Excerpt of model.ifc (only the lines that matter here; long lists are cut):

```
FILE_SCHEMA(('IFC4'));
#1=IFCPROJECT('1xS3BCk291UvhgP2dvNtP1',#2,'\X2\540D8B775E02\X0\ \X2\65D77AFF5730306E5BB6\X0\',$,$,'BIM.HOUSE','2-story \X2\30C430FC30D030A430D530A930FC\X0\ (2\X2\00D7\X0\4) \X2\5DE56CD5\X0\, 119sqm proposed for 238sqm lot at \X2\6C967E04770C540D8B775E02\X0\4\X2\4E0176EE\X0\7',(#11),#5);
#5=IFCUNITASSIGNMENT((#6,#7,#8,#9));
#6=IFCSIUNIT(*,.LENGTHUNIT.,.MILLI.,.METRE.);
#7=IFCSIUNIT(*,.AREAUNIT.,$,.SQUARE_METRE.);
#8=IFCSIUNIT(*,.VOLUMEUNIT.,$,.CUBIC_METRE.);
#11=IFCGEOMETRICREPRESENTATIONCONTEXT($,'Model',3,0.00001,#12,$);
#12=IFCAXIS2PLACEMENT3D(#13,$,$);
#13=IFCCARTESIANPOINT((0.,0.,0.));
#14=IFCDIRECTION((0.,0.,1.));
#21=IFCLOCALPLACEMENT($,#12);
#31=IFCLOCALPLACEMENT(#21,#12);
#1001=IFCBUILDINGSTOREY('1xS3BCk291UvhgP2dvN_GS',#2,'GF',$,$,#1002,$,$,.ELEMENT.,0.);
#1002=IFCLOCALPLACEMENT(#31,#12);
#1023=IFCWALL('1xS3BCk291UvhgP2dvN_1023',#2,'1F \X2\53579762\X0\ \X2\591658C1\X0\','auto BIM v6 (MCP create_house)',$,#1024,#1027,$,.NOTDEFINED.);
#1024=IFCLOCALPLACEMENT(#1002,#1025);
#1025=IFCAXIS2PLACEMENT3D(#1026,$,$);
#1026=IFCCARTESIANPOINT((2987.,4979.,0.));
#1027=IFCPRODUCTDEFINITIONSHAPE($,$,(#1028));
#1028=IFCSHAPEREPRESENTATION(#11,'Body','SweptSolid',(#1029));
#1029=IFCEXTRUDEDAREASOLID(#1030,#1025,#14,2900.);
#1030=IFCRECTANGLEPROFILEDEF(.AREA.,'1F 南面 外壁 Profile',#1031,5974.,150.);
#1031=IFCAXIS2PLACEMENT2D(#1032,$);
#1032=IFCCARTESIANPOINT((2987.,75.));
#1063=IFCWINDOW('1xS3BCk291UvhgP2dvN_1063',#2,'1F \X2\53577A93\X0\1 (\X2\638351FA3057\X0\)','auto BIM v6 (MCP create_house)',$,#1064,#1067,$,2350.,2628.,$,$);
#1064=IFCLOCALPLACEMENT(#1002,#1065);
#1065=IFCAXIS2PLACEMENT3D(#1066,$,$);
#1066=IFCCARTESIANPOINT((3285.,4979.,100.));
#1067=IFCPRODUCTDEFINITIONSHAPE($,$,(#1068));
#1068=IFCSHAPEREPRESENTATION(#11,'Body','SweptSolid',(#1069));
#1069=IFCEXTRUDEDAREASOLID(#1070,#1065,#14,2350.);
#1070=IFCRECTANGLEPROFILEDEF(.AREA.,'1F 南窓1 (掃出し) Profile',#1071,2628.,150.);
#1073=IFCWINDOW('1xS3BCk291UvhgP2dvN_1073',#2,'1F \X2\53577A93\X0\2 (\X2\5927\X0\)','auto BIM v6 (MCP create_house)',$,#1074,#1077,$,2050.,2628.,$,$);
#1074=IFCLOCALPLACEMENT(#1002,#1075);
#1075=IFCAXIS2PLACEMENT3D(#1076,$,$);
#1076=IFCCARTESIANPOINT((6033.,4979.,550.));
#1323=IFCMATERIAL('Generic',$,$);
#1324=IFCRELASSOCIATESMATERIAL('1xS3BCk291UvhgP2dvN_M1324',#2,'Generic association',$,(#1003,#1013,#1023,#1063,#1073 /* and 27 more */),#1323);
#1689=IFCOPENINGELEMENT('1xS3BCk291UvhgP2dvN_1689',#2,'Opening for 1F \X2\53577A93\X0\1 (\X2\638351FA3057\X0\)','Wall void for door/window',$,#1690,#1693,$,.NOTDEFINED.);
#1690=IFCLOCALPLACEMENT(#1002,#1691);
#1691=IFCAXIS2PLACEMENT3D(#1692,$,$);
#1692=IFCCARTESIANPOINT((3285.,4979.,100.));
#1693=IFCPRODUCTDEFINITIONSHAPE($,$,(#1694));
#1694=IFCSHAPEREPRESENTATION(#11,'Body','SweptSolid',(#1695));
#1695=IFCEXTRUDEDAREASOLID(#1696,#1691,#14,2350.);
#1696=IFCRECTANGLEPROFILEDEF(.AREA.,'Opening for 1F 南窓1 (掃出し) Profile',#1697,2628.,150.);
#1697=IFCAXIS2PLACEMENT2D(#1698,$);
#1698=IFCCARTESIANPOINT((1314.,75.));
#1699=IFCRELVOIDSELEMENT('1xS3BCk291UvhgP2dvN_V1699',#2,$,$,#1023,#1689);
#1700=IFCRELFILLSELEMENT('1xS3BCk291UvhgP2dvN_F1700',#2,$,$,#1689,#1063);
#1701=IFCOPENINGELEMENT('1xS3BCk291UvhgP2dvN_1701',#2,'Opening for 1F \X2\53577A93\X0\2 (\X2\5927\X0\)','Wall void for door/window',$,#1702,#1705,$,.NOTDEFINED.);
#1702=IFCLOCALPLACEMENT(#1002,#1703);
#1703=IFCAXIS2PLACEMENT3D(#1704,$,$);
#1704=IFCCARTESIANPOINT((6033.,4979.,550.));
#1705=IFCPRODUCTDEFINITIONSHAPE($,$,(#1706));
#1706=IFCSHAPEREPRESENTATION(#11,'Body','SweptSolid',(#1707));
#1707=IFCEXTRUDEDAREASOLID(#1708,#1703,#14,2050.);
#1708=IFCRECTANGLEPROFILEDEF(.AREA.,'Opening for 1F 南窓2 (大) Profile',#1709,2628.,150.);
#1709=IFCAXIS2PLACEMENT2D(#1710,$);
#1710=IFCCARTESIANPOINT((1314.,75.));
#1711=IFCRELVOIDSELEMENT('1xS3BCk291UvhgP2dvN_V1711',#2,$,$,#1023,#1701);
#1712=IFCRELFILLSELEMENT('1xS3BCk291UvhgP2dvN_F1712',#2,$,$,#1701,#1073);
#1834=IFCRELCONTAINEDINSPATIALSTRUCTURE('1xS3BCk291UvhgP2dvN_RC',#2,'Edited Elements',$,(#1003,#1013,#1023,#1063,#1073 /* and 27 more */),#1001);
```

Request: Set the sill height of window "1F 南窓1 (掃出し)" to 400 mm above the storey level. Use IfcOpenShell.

```python
import numpy as np
import ifcopenshell
import ifcopenshell.api.geometry
import ifcopenshell.geom
import ifcopenshell.util.element
import ifcopenshell.util.placement
import ifcopenshell.util.shape
import ifcopenshell.util.unit

model = ifcopenshell.open("model.ifc")
unit_scale = ifcopenshell.util.unit.calculate_unit_scale(model)

window = model.by_guid("1xS3BCk291UvhgP2dvN_1063")
opening = window.FillsVoids[0].RelatingOpeningElement
storey = ifcopenshell.util.element.get_container(window, ifc_class="IfcBuildingStorey")
level = ifcopenshell.util.placement.get_local_placement(storey.ObjectPlacement)[2, 3]

# The opening's origin need not be at the sill, so measure its lowest point.
shape = ifcopenshell.geom.create_shape(ifcopenshell.geom.settings(), opening)
bottom = ifcopenshell.util.shape.get_shape_bottom_elevation(shape, shape.geometry) / unit_scale
dz = level + 0.4 / unit_scale - bottom

shift = np.array([0.0, 0.0, dz])
# The window is not placed relative to its opening, so move both.
for product in (opening, window):
    matrix = ifcopenshell.util.placement.get_local_placement(product.ObjectPlacement)
    matrix[:3, 3] += shift
    ifcopenshell.api.geometry.edit_object_placement(model, product=product, matrix=matrix, is_si=False)

print(f"moved by {dz * unit_scale:+.3f} m")

model.write("model_v2.ifc")
```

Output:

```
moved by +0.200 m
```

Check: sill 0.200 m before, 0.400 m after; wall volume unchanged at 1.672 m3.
